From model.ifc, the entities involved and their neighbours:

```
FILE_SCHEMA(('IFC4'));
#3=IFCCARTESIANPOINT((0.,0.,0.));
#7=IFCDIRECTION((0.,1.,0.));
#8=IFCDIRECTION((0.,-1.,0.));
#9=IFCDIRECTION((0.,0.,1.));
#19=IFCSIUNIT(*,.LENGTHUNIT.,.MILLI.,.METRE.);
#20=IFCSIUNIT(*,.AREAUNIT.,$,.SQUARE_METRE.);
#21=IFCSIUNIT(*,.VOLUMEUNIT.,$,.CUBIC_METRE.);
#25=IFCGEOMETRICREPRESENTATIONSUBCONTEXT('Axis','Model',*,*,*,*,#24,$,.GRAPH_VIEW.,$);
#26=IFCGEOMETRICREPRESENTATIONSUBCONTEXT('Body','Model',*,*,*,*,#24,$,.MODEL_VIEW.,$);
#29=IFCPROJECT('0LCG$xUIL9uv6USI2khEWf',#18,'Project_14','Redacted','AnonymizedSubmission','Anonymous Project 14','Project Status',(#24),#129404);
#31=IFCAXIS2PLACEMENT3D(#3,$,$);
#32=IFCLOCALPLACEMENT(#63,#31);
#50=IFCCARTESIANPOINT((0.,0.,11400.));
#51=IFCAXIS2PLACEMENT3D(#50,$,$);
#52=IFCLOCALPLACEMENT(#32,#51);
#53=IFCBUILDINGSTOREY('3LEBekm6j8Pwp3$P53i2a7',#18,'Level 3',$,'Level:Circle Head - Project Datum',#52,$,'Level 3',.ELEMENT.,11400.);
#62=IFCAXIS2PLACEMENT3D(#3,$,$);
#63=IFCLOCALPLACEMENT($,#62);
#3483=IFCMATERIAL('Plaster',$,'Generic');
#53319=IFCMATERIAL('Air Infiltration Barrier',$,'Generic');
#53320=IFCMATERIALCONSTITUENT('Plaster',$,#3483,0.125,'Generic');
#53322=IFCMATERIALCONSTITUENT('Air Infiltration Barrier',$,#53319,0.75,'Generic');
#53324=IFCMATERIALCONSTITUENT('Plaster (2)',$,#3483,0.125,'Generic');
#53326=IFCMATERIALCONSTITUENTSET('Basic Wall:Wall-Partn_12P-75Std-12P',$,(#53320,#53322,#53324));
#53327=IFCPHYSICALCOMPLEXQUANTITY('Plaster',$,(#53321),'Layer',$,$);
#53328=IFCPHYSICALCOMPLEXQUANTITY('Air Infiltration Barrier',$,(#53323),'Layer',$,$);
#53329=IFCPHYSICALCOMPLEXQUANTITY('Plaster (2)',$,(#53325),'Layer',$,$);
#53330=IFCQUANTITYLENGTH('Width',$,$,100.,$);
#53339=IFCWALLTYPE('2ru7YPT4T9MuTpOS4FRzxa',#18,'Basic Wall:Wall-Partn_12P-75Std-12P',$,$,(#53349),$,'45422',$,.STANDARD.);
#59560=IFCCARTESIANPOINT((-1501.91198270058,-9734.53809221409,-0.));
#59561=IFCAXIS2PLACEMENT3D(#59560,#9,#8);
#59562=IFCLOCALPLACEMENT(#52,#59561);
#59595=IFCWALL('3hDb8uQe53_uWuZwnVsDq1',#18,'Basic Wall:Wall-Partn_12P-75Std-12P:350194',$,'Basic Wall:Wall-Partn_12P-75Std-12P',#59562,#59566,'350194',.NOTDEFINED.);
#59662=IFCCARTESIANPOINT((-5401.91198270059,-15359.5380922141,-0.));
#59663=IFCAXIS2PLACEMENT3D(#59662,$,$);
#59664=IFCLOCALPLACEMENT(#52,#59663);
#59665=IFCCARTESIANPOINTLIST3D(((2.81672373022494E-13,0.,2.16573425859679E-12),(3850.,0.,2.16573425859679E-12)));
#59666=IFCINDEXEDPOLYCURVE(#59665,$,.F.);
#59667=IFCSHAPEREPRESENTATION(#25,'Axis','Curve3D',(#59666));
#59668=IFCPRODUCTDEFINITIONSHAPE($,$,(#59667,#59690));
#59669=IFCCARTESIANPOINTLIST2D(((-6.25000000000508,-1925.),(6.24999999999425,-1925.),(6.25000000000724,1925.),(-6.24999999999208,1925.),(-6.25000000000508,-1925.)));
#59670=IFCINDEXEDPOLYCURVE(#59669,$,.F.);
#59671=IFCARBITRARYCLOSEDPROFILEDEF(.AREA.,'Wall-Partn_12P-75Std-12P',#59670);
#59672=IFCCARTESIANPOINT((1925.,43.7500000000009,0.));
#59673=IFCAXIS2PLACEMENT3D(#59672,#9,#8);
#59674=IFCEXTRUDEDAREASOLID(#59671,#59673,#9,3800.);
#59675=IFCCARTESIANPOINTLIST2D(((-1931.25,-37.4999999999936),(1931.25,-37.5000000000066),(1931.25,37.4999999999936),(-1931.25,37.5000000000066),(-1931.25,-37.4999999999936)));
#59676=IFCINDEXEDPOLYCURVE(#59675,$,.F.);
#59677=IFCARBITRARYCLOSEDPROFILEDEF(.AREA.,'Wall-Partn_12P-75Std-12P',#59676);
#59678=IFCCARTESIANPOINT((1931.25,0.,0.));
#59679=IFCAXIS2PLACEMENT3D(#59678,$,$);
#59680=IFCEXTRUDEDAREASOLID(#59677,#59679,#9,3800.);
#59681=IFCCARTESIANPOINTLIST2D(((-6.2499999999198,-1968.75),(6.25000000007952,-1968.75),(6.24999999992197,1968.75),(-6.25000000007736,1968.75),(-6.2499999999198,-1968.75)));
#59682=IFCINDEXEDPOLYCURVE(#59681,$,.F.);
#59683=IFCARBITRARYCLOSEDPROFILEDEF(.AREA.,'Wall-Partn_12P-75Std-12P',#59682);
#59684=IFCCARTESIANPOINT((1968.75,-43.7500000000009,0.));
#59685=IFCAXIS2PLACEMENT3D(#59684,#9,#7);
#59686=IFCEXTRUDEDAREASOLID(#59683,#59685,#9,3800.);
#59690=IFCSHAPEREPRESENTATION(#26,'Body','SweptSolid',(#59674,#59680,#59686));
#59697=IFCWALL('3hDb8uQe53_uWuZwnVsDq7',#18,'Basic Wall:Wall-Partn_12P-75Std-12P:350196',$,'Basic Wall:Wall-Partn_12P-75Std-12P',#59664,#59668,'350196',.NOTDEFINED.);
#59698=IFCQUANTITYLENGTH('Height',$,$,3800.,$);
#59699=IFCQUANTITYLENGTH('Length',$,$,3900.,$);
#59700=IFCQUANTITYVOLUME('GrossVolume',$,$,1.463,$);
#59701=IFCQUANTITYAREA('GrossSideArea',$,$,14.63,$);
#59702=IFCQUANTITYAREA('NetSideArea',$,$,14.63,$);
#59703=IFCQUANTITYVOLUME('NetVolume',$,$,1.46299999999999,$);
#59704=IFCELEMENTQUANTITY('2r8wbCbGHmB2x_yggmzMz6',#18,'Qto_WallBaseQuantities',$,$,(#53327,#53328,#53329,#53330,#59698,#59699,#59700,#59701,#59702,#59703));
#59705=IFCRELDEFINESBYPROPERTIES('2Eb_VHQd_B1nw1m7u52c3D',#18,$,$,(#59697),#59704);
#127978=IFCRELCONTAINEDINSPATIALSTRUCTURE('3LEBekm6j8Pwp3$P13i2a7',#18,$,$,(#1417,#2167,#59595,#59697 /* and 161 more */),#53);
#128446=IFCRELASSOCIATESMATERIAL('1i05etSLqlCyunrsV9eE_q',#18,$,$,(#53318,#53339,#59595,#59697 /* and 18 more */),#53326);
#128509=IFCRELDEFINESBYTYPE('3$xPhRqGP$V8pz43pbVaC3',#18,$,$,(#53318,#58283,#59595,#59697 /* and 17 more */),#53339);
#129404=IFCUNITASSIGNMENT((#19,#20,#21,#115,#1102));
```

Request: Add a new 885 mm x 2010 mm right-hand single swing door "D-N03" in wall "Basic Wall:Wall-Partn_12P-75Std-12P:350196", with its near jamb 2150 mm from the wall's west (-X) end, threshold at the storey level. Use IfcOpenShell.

```python
import numpy as np
import ifcopenshell
import ifcopenshell.api.feature
import ifcopenshell.api.geometry
import ifcopenshell.api.pset
import ifcopenshell.api.root
import ifcopenshell.api.spatial
import ifcopenshell.geom
import ifcopenshell.util.element
import ifcopenshell.util.placement
import ifcopenshell.util.representation
import ifcopenshell.util.shape
import ifcopenshell.util.unit

model = ifcopenshell.open("model.ifc")
unit_scale = ifcopenshell.util.unit.calculate_unit_scale(model)
area_scale = ifcopenshell.util.unit.calculate_unit_scale(model, "AREAUNIT")
volume_scale = ifcopenshell.util.unit.calculate_unit_scale(model, "VOLUMEUNIT")
settings = ifcopenshell.geom.settings()


def volume(element):
    """Net volume in cubic metres, openings subtracted."""
    shape = ifcopenshell.geom.create_shape(settings, element)
    return ifcopenshell.util.shape.get_volume(shape.geometry)


wall = model.by_id(59697)
storey = ifcopenshell.util.element.get_container(wall, ifc_class="IfcBuildingStorey")
context = ifcopenshell.util.representation.get_context(model, "Model", "Body", "MODEL_VIEW")
before = volume(wall)

width, height, from_end, sill = 0.885, 2.01, 2.15, 0.0  # metres

# The wall runs along its own X axis, and the end named is its -X end.
wall_shape = ifcopenshell.geom.create_shape(settings, wall)
x, y, z = ifcopenshell.util.shape.get_vertices(wall_shape.geometry).T
start = x.min() + from_end
face, thickness = float(y.min()), float(y.max() - y.min())
wall_matrix = ifcopenshell.util.placement.get_local_placement(wall.ObjectPlacement)
level = ifcopenshell.util.placement.get_local_placement(storey.ObjectPlacement)[2, 3]


def in_wall(x, y):
    """Placement at x, y metres in the wall's axes, at sill height."""
    matrix = wall_matrix.copy()
    matrix[:, 3] = wall_matrix @ np.array([x / unit_scale, y / unit_scale, 0.0, 1.0])
    matrix[2, 3] = level + sill / unit_scale
    return matrix


# Opening: a box that overshoots both wall faces by 50 mm.
opening = ifcopenshell.api.root.create_entity(model, ifc_class="IfcOpeningElement", predefined_type="OPENING")
box = ifcopenshell.api.geometry.add_wall_representation(
    model, context=context, length=width, height=height, thickness=thickness + 0.1
)
ifcopenshell.api.geometry.assign_representation(model, product=opening, representation=box)
ifcopenshell.api.geometry.edit_object_placement(model, product=opening, matrix=in_wall(start, face - 0.05), is_si=False)
ifcopenshell.api.feature.add_feature(model, feature=opening, element=wall)

door = ifcopenshell.api.root.create_entity(model, ifc_class="IfcDoor", name="D-N03", predefined_type="DOOR")
door.OverallWidth, door.OverallHeight = width / unit_scale, height / unit_scale
door.OperationType = "SINGLE_SWING_RIGHT"
body = ifcopenshell.api.geometry.add_door_representation(
    model,
    context=context,
    overall_width=door.OverallWidth,
    overall_height=door.OverallHeight,
    operation_type="SINGLE_SWING_RIGHT",
    lining_properties={"LiningDepth": thickness / unit_scale, "ThresholdDepth": thickness / unit_scale},
)
ifcopenshell.api.geometry.assign_representation(model, product=door, representation=body)
ifcopenshell.api.spatial.assign_container(model, products=[door], relating_structure=storey)
ifcopenshell.api.feature.add_filling(model, opening=opening, element=door)

# The lining spans the wall, so the door starts at the wall face.
ifcopenshell.api.geometry.edit_object_placement(model, product=door, matrix=in_wall(start, face), is_si=False)

after = volume(wall)

# Update the wall's stored quantities.
qto = model.by_id(ifcopenshell.util.element.get_pset(wall, "Qto_WallBaseQuantities", should_inherit=False)["id"])
ifcopenshell.api.pset.edit_qto(model, qto=qto, properties={
    "NetSideArea": after / thickness / area_scale,
    "NetVolume": after / volume_scale,
})

print(f"wall volume {before:.3f} -> {after:.3f} m3")

model.write("model-out.ifc")
```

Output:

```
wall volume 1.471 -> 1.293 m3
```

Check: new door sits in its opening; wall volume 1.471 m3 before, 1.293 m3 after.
